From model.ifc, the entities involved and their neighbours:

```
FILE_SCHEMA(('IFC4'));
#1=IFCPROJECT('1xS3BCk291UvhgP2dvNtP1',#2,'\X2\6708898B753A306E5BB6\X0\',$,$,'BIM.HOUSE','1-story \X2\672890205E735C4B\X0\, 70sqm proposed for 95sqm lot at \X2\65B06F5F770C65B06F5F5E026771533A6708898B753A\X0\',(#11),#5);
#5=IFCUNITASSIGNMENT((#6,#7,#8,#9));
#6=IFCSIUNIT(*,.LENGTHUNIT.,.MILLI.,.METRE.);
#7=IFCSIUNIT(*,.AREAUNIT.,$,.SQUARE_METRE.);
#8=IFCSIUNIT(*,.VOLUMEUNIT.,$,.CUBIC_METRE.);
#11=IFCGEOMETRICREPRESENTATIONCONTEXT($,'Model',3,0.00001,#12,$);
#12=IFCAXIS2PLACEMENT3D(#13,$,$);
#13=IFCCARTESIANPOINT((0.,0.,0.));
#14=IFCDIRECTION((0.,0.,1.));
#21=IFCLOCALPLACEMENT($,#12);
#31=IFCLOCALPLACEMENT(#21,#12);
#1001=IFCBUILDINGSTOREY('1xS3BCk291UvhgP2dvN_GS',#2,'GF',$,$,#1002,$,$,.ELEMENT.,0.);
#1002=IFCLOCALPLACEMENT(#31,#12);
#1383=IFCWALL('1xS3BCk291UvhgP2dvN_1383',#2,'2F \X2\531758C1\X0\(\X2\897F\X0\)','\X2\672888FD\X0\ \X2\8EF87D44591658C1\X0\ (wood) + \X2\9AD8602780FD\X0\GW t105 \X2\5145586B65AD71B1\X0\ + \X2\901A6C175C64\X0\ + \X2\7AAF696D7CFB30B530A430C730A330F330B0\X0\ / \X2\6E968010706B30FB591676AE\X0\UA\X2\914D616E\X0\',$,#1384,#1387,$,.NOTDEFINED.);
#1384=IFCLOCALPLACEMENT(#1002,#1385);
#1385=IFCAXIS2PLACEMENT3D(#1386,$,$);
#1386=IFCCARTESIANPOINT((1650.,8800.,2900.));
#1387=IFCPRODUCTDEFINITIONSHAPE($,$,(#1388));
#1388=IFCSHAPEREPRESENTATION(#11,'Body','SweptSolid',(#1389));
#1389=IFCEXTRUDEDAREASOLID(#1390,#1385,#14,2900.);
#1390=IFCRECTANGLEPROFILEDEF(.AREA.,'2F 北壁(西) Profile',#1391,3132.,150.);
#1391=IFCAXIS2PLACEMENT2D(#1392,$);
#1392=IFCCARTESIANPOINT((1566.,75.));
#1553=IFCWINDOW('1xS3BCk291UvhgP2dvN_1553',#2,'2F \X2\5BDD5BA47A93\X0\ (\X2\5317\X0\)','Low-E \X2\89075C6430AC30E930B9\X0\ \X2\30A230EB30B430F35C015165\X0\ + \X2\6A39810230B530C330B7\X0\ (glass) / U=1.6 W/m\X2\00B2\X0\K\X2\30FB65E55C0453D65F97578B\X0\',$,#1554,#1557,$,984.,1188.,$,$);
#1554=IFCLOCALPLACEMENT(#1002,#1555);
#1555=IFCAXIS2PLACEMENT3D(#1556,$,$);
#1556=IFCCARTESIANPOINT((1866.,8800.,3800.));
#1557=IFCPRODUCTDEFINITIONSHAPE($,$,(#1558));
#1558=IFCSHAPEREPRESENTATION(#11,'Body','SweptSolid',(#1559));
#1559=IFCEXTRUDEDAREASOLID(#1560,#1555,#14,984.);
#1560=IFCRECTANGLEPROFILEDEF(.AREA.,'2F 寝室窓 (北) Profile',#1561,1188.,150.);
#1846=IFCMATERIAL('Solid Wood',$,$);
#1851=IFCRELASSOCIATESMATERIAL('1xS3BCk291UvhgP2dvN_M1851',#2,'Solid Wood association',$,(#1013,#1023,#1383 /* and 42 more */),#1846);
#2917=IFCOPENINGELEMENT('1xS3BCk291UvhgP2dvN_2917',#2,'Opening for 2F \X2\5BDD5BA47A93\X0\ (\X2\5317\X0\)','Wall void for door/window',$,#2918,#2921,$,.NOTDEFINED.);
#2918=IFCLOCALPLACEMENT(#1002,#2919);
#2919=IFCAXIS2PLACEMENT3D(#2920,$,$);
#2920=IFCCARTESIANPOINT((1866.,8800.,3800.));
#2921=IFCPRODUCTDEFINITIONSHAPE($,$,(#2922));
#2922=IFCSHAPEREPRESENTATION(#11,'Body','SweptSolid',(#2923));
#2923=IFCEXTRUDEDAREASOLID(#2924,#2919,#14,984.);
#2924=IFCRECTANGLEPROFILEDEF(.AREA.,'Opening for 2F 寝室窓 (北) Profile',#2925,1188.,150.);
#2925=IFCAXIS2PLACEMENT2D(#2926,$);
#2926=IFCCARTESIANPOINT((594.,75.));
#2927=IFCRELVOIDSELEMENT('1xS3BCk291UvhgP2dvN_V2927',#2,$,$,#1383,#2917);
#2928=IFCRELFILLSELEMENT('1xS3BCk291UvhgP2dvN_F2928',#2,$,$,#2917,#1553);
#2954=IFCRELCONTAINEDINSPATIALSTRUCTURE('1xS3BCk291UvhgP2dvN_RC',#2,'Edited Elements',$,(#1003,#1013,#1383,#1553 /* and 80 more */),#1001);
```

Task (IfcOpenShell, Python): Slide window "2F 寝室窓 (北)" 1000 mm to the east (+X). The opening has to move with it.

```python
import ifcopenshell
import ifcopenshell.api.geometry
import ifcopenshell.util.placement
import ifcopenshell.util.unit

model = ifcopenshell.open("model.ifc")
unit_scale = ifcopenshell.util.unit.calculate_unit_scale(model)

window = model.by_guid("1xS3BCk291UvhgP2dvN_1553")
opening = window.FillsVoids[0].RelatingOpeningElement
wall = opening.VoidsElements[0].RelatingBuildingElement

wall_matrix = ifcopenshell.util.placement.get_local_placement(wall.ObjectPlacement)
shift = wall_matrix[:3, 0] * 1 / unit_scale
before = ifcopenshell.util.placement.get_local_placement(window.ObjectPlacement)[:3, 3].copy()

# The window is not placed relative to its opening, so move both.
for product in (opening, window):
    matrix = ifcopenshell.util.placement.get_local_placement(product.ObjectPlacement)
    matrix[:3, 3] += shift
    ifcopenshell.api.geometry.edit_object_placement(model, product=product, matrix=matrix, is_si=False)

after = ifcopenshell.util.placement.get_local_placement(window.ObjectPlacement)[:3, 3]
print("window moved by", (after - before).round(3) + 0.0)

model.write("model-out.ifc")
```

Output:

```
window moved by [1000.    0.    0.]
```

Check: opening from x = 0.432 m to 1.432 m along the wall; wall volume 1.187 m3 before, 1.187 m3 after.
